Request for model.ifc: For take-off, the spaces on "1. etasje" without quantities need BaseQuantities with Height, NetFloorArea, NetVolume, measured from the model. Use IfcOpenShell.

First a look at what the model holds.

```python
import ifcopenshell
import ifcopenshell.util.element
import ifcopenshell.util.unit

model = ifcopenshell.open("model.ifc")
print(model.schema)
for unit_type in ("LENGTHUNIT", "AREAUNIT", "VOLUMEUNIT"):
    print(unit_type, ifcopenshell.util.unit.calculate_unit_scale(model, unit_type))
storey = next(s for s in model.by_type("IfcBuildingStorey") if s.Name == "1. etasje")
spaces = [e for e in ifcopenshell.util.element.get_decomposition(storey) if e.is_a("IfcSpace")]
for e in sorted(spaces, key=lambda e: e.id()):
    print(e.id(), e.is_a(), e.Name, list(ifcopenshell.util.element.get_psets(e, qtos_only=True)), sep=" | ")
```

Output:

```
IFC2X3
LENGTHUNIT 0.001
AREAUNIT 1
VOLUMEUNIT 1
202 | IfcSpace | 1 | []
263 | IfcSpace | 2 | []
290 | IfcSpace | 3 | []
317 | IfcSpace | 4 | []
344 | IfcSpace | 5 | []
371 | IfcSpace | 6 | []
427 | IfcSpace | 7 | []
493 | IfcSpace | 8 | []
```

```python
import ifcopenshell
import ifcopenshell.api.pset
import ifcopenshell.geom
import ifcopenshell.util.element
import ifcopenshell.util.shape
import ifcopenshell.util.unit

model = ifcopenshell.open("model.ifc")
unit_scale = ifcopenshell.util.unit.calculate_unit_scale(model)
area_scale = ifcopenshell.util.unit.calculate_unit_scale(model, "AREAUNIT")
volume_scale = ifcopenshell.util.unit.calculate_unit_scale(model, "VOLUMEUNIT")
settings = ifcopenshell.geom.settings()

storey = next(s for s in model.by_type("IfcBuildingStorey") if s.Name == "1. etasje")
spaces = [e for e in ifcopenshell.util.element.get_decomposition(storey) if e.is_a("IfcSpace")]

for e in sorted(spaces, key=lambda e: e.id()):
    if ifcopenshell.util.element.get_psets(e, qtos_only=True, should_inherit=False):
        continue
    # Geometry comes back in metres, in the element's own axes.
    shape = ifcopenshell.geom.create_shape(settings, e)
    values = {
        "Height": ifcopenshell.util.shape.get_z(shape.geometry) / unit_scale,
        "NetFloorArea": ifcopenshell.util.shape.get_footprint_area(shape.geometry) / area_scale,
        "NetVolume": ifcopenshell.util.shape.get_volume(shape.geometry) / volume_scale,
    }
    qto = ifcopenshell.api.pset.add_qto(model, product=e, name="BaseQuantities")
    ifcopenshell.api.pset.edit_qto(model, qto=qto, properties=values)
    print(e.id(), {k: round(v, 3) for k, v in values.items()})

model.write("model_v2.ifc")
```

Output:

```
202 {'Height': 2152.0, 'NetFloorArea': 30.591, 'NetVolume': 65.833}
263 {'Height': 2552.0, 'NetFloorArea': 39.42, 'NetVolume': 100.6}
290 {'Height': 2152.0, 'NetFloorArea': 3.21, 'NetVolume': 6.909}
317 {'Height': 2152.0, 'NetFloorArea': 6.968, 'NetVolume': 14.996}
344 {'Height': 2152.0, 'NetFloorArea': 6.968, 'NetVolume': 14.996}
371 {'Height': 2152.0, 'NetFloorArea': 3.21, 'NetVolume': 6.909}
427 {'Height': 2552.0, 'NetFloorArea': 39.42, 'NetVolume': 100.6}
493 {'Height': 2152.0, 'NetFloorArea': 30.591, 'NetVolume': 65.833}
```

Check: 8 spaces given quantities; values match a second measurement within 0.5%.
